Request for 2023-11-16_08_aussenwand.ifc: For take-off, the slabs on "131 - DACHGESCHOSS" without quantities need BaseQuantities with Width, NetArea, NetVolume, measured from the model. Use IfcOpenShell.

First a look at what the model holds.

```python
import ifcopenshell
import ifcopenshell.util.element
import ifcopenshell.util.unit

model = ifcopenshell.open("2023-11-16_08_aussenwand.ifc")
print(model.schema)
for unit_type in ("LENGTHUNIT", "AREAUNIT", "VOLUMEUNIT"):
    print(unit_type, ifcopenshell.util.unit.calculate_unit_scale(model, unit_type))
storey = next(s for s in model.by_type("IfcBuildingStorey") if s.Name == "131 - DACHGESCHOSS")
slabs = [e for e in ifcopenshell.util.element.get_decomposition(storey) if e.is_a("IfcSlab")]
for e in sorted(slabs, key=lambda e: e.id()):
    print(e.id(), e.is_a(), e.Name, list(ifcopenshell.util.element.get_psets(e, qtos_only=True)), sep=" | ")
```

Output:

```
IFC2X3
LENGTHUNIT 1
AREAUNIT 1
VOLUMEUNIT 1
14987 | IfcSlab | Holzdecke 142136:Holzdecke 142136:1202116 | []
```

```python
import ifcopenshell
import ifcopenshell.api.pset
import ifcopenshell.geom
import ifcopenshell.util.element
import ifcopenshell.util.shape
import ifcopenshell.util.unit

model = ifcopenshell.open("2023-11-16_08_aussenwand.ifc")
unit_scale = ifcopenshell.util.unit.calculate_unit_scale(model)
area_scale = ifcopenshell.util.unit.calculate_unit_scale(model, "AREAUNIT")
volume_scale = ifcopenshell.util.unit.calculate_unit_scale(model, "VOLUMEUNIT")
settings = ifcopenshell.geom.settings()

storey = next(s for s in model.by_type("IfcBuildingStorey") if s.Name == "131 - DACHGESCHOSS")
slabs = [e for e in ifcopenshell.util.element.get_decomposition(storey) if e.is_a("IfcSlab")]

for e in sorted(slabs, key=lambda e: e.id()):
    if ifcopenshell.util.element.get_psets(e, qtos_only=True, should_inherit=False):
        continue
    # Geometry comes back in metres, in the element's own axes.
    shape = ifcopenshell.geom.create_shape(settings, e)
    values = {
        "Width": ifcopenshell.util.shape.get_z(shape.geometry) / unit_scale,
        "NetArea": ifcopenshell.util.shape.get_footprint_area(shape.geometry) / area_scale,
        "NetVolume": ifcopenshell.util.shape.get_volume(shape.geometry) / volume_scale,
    }
    qto = ifcopenshell.api.pset.add_qto(model, product=e, name="BaseQuantities")
    ifcopenshell.api.pset.edit_qto(model, qto=qto, properties=values)
    print(e.id(), {k: round(v, 3) for k, v in values.items()})

model.write("2023-11-16_08_aussenwand_updated.ifc")
```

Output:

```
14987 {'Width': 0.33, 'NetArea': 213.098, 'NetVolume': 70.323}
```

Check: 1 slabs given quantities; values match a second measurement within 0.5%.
